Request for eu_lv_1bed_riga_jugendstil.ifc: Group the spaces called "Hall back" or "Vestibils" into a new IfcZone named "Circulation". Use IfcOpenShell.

First a look at what the model holds.

```python
import ifcopenshell

model = ifcopenshell.open("eu_lv_1bed_riga_jugendstil.ifc")
print(model.schema)
seen = {}
for space in model.by_type("IfcSpace"):
    seen[space.LongName] = seen.get(space.LongName, 0) + 1
for name, count in sorted(seen.items(), key=str):
    print(count, "x", name)
print("zones:", [z.Name for z in model.by_type("IfcZone")][:20])
```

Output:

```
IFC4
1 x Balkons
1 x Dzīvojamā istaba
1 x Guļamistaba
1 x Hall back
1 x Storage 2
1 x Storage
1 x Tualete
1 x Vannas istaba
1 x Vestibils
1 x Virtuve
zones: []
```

```python
import ifcopenshell
import ifcopenshell.api.group
import ifcopenshell.api.root

model = ifcopenshell.open("eu_lv_1bed_riga_jugendstil.ifc")

names = {"Hall back", "Vestibils"}
spaces = [s for s in model.by_type("IfcSpace") if s.LongName in names]

zone = ifcopenshell.api.root.create_entity(model, ifc_class="IfcZone", name="Circulation")
ifcopenshell.api.group.assign_group(model, products=spaces, group=zone)
print(len(spaces), "spaces in", zone.Name)

model.write("eu_lv_1bed_riga_jugendstil_v2.ifc")
```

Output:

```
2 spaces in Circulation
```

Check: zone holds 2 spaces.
